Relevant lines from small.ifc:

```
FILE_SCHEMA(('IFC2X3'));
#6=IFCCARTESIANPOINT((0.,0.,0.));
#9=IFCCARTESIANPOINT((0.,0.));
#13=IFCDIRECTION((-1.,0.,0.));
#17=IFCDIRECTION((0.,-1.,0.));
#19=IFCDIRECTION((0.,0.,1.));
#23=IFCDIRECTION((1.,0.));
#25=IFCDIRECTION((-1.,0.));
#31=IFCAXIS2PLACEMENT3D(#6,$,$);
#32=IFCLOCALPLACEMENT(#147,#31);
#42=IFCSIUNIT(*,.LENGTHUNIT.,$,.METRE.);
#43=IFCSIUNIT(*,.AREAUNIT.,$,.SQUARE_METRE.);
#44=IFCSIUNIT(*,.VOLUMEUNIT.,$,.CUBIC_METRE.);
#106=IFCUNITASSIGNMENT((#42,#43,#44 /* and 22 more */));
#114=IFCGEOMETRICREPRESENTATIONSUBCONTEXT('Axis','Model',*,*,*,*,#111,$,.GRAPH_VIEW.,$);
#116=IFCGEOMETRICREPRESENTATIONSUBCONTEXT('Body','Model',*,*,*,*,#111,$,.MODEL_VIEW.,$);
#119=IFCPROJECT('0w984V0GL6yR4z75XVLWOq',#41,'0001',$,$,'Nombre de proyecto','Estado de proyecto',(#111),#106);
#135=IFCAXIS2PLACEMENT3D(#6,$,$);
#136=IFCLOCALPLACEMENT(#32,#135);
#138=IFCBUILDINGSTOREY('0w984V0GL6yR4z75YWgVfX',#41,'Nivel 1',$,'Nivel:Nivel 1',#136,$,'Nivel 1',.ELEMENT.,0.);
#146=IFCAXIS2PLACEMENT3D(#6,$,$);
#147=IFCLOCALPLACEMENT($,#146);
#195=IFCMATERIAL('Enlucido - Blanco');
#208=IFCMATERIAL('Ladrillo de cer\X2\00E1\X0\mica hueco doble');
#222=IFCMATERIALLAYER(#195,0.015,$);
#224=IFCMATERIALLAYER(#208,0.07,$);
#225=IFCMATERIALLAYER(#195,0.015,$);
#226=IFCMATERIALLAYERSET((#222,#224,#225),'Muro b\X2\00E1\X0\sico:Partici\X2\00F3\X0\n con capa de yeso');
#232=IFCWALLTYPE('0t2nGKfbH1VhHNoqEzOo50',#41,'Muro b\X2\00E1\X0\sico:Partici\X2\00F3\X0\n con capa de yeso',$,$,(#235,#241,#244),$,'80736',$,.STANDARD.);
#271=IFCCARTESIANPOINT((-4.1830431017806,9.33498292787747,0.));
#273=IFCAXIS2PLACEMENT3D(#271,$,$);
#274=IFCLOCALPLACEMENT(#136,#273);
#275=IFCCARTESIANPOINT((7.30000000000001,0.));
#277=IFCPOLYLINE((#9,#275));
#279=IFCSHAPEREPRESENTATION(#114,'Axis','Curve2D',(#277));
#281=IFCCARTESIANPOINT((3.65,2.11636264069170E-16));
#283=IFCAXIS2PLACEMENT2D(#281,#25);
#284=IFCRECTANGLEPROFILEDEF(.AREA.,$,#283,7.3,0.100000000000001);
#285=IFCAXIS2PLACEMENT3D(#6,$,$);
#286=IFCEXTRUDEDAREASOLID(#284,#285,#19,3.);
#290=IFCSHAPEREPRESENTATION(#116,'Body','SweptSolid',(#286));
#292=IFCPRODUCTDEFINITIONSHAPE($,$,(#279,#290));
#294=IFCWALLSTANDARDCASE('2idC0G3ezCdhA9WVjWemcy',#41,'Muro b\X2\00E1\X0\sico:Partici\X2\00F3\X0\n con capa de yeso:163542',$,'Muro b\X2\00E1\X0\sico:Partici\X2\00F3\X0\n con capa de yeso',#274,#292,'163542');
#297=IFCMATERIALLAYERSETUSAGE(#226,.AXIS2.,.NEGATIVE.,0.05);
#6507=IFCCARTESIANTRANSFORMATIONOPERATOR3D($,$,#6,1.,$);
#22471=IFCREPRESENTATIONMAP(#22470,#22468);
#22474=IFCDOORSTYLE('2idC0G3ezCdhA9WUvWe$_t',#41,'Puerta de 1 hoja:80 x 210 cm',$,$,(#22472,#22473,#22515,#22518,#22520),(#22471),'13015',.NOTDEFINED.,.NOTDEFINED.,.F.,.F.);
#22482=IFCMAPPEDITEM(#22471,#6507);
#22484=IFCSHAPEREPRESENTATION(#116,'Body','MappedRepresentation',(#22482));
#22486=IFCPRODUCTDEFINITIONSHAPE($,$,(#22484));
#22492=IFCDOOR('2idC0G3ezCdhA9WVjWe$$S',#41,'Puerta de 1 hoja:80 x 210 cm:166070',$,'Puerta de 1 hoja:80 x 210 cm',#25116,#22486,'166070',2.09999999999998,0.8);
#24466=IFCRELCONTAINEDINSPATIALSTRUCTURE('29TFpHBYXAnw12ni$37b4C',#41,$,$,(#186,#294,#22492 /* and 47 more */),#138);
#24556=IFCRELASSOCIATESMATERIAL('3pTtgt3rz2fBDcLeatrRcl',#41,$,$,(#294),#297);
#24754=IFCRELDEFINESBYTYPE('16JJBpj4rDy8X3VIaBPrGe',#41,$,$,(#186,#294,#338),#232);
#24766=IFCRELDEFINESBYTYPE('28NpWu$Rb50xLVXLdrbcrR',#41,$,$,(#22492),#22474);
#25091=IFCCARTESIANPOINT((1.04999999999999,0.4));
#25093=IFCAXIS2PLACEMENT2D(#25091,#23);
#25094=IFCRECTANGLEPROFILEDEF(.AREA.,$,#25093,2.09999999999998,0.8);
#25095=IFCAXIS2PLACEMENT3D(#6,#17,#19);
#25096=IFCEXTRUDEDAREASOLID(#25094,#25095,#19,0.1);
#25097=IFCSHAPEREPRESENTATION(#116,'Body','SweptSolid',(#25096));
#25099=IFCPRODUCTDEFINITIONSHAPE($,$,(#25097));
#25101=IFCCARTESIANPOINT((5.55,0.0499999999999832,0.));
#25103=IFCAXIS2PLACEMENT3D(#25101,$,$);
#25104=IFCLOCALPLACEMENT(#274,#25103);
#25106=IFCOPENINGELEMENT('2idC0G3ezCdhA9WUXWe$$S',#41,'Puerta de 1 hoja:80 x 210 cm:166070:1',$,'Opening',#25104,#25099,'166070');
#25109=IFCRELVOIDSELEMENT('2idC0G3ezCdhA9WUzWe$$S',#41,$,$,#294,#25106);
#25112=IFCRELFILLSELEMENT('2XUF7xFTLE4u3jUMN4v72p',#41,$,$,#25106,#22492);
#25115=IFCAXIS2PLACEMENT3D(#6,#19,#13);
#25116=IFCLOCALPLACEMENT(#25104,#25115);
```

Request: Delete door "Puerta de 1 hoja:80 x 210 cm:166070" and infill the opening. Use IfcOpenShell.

```python
import ifcopenshell
import ifcopenshell.api.feature
import ifcopenshell.api.root
import ifcopenshell.geom
import ifcopenshell.util.shape

model = ifcopenshell.open("small.ifc")
settings = ifcopenshell.geom.settings()


def volume(element):
    """Net volume in cubic metres, openings subtracted."""
    shape = ifcopenshell.geom.create_shape(settings, element)
    return ifcopenshell.util.shape.get_volume(shape.geometry)


door = model.by_guid("2idC0G3ezCdhA9WVjWe$$S")
opening = door.FillsVoids[0].RelatingOpeningElement
wall = opening.VoidsElements[0].RelatingBuildingElement
before = volume(wall)

ifcopenshell.api.root.remove_product(model, product=door)
ifcopenshell.api.feature.remove_feature(model, feature=opening)

after = volume(wall)

print(f"wall volume {before:.3f} -> {after:.3f} m3")

model.write("small_rev.ifc")
```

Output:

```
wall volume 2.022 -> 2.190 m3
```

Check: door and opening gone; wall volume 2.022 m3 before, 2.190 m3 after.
